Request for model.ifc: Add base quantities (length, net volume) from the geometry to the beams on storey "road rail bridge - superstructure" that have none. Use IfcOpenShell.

First a look at what the model holds.

```python
import ifcopenshell
import ifcopenshell.util.element
import ifcopenshell.util.unit

model = ifcopenshell.open("model.ifc")
print(model.schema)
for unit_type in ("LENGTHUNIT", "AREAUNIT", "VOLUMEUNIT"):
    print(unit_type, ifcopenshell.util.unit.calculate_unit_scale(model, unit_type))
storey = next(s for s in model.by_type("IfcBuildingStorey") if s.Name == "road rail bridge - superstructure")
beams = [e for e in ifcopenshell.util.element.get_decomposition(storey) if e.is_a("IfcBeam")]
for e in sorted(beams, key=lambda e: e.id()):
    print(e.id(), e.is_a(), e.Name, list(ifcopenshell.util.element.get_psets(e, qtos_only=True)), sep=" | ")
```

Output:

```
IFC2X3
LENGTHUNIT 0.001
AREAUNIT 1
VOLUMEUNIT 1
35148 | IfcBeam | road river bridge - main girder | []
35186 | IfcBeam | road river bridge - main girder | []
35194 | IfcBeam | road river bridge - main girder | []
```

```python
import ifcopenshell
import ifcopenshell.api.pset
import ifcopenshell.geom
import ifcopenshell.util.element
import ifcopenshell.util.shape
import ifcopenshell.util.unit

model = ifcopenshell.open("model.ifc")
unit_scale = ifcopenshell.util.unit.calculate_unit_scale(model)
volume_scale = ifcopenshell.util.unit.calculate_unit_scale(model, "VOLUMEUNIT")
settings = ifcopenshell.geom.settings()

storey = next(s for s in model.by_type("IfcBuildingStorey") if s.Name == "road rail bridge - superstructure")
beams = [e for e in ifcopenshell.util.element.get_decomposition(storey) if e.is_a("IfcBeam")]

for e in sorted(beams, key=lambda e: e.id()):
    if ifcopenshell.util.element.get_psets(e, qtos_only=True, should_inherit=False):
        continue
    # Geometry comes back in metres, in the element's own axes.
    shape = ifcopenshell.geom.create_shape(settings, e)
    values = {
        "Length": ifcopenshell.util.shape.get_max_xyz(shape.geometry) / unit_scale,
        "NetVolume": ifcopenshell.util.shape.get_volume(shape.geometry) / volume_scale,
    }
    qto = ifcopenshell.api.pset.add_qto(model, product=e, name="BaseQuantities")
    ifcopenshell.api.pset.edit_qto(model, qto=qto, properties=values)
    print(e.id(), {k: round(v, 3) for k, v in values.items()})

model.write("model_rev.ifc")
```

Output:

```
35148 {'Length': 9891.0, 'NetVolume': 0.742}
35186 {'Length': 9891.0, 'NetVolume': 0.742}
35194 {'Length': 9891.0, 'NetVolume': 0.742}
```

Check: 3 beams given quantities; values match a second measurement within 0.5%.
